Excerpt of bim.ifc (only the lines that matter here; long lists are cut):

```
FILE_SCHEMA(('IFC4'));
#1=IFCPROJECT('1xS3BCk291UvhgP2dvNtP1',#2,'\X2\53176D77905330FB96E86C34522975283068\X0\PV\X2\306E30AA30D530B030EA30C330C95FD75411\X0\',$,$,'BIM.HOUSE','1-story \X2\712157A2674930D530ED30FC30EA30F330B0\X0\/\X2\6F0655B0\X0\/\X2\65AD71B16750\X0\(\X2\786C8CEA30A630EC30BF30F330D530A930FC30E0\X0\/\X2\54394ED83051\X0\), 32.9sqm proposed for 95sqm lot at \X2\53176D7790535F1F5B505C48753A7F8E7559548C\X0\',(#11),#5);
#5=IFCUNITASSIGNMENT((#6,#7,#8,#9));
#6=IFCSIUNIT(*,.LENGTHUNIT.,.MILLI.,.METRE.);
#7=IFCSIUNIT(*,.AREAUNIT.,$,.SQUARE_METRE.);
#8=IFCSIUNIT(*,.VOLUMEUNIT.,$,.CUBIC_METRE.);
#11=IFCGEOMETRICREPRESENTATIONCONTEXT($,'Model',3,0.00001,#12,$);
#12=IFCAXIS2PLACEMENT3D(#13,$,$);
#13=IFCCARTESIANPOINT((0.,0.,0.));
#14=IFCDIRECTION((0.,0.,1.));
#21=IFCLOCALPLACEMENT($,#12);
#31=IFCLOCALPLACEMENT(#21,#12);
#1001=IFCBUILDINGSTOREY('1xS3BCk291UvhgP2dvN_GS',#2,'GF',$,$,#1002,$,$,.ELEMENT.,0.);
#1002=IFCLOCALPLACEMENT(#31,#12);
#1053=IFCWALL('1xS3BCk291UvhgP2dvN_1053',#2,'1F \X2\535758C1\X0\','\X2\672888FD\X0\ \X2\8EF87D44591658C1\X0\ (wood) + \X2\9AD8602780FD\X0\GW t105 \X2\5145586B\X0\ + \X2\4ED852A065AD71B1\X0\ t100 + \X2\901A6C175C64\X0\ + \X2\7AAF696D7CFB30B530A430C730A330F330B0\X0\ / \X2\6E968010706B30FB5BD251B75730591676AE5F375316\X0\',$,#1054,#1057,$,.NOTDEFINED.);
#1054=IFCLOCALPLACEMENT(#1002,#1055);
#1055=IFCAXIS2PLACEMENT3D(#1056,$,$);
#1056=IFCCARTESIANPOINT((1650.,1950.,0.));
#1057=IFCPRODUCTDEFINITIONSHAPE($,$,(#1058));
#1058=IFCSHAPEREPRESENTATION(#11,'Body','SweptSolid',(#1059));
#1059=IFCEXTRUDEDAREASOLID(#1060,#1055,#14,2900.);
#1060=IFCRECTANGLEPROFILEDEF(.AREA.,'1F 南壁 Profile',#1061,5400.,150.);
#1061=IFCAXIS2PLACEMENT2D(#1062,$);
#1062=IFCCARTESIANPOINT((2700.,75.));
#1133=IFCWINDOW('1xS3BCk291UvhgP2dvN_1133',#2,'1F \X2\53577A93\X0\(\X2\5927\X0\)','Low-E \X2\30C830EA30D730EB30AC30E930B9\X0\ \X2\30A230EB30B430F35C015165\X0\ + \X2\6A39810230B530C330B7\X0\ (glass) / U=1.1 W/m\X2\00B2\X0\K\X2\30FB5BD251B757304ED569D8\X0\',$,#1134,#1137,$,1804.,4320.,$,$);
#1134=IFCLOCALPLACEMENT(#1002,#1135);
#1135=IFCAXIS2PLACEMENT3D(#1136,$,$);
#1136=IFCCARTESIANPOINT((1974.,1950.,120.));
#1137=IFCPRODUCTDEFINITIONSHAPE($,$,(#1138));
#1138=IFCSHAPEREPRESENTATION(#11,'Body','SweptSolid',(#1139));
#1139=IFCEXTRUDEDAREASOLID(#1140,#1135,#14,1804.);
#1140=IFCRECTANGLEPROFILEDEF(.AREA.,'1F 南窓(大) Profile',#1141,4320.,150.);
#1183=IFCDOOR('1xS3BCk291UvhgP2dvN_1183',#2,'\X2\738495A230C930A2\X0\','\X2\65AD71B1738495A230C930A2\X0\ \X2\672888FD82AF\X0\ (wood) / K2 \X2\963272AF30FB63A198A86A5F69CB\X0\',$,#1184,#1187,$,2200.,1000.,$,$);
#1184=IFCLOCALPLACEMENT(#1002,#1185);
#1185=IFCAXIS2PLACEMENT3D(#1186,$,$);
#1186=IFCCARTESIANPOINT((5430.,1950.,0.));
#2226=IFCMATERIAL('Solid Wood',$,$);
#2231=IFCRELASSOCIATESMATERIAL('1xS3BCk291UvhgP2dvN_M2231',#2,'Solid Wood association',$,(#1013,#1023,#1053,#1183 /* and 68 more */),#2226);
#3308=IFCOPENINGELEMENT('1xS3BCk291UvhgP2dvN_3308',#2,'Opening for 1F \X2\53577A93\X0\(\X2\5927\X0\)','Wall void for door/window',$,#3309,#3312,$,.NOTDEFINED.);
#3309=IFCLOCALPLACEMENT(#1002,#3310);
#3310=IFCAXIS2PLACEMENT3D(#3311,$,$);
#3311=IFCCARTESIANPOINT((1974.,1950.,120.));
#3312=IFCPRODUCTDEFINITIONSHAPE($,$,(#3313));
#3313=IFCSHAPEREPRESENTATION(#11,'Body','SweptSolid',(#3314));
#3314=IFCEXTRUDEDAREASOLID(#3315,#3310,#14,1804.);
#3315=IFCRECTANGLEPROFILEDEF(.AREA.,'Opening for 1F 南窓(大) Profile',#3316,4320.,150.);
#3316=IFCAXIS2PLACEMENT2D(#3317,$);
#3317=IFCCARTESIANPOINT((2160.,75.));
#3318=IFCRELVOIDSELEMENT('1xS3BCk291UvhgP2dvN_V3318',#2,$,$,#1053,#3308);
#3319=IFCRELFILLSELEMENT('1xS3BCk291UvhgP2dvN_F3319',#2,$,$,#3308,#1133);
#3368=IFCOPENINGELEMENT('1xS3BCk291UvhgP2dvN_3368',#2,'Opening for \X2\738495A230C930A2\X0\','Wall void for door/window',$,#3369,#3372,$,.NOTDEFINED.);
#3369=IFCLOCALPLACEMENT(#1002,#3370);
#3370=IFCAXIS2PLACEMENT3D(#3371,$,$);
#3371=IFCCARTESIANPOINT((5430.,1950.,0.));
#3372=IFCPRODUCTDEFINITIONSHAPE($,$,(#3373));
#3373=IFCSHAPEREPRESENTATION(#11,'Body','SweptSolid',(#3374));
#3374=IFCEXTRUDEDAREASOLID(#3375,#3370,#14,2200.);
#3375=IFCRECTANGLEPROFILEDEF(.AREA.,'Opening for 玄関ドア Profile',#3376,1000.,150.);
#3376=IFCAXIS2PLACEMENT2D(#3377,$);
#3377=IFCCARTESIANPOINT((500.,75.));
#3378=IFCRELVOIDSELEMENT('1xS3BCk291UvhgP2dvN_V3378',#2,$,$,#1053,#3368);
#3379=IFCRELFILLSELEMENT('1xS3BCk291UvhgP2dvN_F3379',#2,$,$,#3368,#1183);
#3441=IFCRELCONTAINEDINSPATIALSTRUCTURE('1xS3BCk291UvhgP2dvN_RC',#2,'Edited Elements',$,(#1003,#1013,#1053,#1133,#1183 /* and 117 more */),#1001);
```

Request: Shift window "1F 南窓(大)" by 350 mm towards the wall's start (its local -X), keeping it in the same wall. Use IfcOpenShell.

```python
import ifcopenshell
import ifcopenshell.api.geometry
import ifcopenshell.util.placement
import ifcopenshell.util.unit

model = ifcopenshell.open("bim.ifc")
unit_scale = ifcopenshell.util.unit.calculate_unit_scale(model)

window = model.by_guid("1xS3BCk291UvhgP2dvN_1133")
opening = window.FillsVoids[0].RelatingOpeningElement
wall = opening.VoidsElements[0].RelatingBuildingElement

wall_matrix = ifcopenshell.util.placement.get_local_placement(wall.ObjectPlacement)
shift = wall_matrix[:3, 0] * -0.35 / unit_scale
before = ifcopenshell.util.placement.get_local_placement(window.ObjectPlacement)[:3, 3].copy()

# The window is not placed relative to its opening, so move both.
for product in (opening, window):
    matrix = ifcopenshell.util.placement.get_local_placement(product.ObjectPlacement)
    matrix[:3, 3] += shift
    ifcopenshell.api.geometry.edit_object_placement(model, product=product, matrix=matrix, is_si=False)

after = ifcopenshell.util.placement.get_local_placement(window.ObjectPlacement)[:3, 3]
print("window moved by", (after - before).round(3) + 0.0)

model.write("bim-out.ifc")
```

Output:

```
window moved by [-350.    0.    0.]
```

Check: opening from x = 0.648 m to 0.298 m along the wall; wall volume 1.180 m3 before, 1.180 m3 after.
